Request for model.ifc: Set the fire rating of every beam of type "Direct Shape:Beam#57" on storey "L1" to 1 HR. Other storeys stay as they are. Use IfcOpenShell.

First a look at what the model holds.

```python
import ifcopenshell
import ifcopenshell.util.element

model = ifcopenshell.open("model.ifc")
print(model.schema)
storey = next(s for s in model.by_type("IfcBuildingStorey") if s.Name == "L1")
beams = [e for e in ifcopenshell.util.element.get_decomposition(storey) if e.is_a("IfcBeam")]
seen = {}
for e in beams:
    element_type = ifcopenshell.util.element.get_type(e)
    key = (element_type.Name if element_type != e and element_type else None, ifcopenshell.util.element.get_pset(e, "Pset_BeamCommon", "FireRating"))
    seen[key] = seen.get(key, 0) + 1
for (name, value), count in sorted(seen.items(), key=str):
    print(count, "x", name, "|", value)
```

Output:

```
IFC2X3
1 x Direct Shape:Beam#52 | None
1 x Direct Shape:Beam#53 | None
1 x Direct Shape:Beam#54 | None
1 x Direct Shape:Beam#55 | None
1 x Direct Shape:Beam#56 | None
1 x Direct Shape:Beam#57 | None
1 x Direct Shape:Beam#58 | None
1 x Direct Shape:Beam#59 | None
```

```python
import ifcopenshell
import ifcopenshell.api.pset
import ifcopenshell.util.element

model = ifcopenshell.open("model.ifc")

storey = next(s for s in model.by_type("IfcBuildingStorey") if s.Name == "L1")
beams = [e for e in ifcopenshell.util.element.get_decomposition(storey) if e.is_a("IfcBeam")]

count = 0
for e in beams:
    element_type = ifcopenshell.util.element.get_type(e)
    if element_type in (None, e) or element_type.Name != "Direct Shape:Beam#57":
        continue
    # add_pset returns the element's existing set when there is one.
    pset = ifcopenshell.api.pset.add_pset(model, product=e, name="Pset_BeamCommon")
    ifcopenshell.api.pset.edit_pset(model, pset=pset, properties={"FireRating": "1 HR"})
    count += 1

print(count, "beams updated")

model.write("model-out.ifc")
```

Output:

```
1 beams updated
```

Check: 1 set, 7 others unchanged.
